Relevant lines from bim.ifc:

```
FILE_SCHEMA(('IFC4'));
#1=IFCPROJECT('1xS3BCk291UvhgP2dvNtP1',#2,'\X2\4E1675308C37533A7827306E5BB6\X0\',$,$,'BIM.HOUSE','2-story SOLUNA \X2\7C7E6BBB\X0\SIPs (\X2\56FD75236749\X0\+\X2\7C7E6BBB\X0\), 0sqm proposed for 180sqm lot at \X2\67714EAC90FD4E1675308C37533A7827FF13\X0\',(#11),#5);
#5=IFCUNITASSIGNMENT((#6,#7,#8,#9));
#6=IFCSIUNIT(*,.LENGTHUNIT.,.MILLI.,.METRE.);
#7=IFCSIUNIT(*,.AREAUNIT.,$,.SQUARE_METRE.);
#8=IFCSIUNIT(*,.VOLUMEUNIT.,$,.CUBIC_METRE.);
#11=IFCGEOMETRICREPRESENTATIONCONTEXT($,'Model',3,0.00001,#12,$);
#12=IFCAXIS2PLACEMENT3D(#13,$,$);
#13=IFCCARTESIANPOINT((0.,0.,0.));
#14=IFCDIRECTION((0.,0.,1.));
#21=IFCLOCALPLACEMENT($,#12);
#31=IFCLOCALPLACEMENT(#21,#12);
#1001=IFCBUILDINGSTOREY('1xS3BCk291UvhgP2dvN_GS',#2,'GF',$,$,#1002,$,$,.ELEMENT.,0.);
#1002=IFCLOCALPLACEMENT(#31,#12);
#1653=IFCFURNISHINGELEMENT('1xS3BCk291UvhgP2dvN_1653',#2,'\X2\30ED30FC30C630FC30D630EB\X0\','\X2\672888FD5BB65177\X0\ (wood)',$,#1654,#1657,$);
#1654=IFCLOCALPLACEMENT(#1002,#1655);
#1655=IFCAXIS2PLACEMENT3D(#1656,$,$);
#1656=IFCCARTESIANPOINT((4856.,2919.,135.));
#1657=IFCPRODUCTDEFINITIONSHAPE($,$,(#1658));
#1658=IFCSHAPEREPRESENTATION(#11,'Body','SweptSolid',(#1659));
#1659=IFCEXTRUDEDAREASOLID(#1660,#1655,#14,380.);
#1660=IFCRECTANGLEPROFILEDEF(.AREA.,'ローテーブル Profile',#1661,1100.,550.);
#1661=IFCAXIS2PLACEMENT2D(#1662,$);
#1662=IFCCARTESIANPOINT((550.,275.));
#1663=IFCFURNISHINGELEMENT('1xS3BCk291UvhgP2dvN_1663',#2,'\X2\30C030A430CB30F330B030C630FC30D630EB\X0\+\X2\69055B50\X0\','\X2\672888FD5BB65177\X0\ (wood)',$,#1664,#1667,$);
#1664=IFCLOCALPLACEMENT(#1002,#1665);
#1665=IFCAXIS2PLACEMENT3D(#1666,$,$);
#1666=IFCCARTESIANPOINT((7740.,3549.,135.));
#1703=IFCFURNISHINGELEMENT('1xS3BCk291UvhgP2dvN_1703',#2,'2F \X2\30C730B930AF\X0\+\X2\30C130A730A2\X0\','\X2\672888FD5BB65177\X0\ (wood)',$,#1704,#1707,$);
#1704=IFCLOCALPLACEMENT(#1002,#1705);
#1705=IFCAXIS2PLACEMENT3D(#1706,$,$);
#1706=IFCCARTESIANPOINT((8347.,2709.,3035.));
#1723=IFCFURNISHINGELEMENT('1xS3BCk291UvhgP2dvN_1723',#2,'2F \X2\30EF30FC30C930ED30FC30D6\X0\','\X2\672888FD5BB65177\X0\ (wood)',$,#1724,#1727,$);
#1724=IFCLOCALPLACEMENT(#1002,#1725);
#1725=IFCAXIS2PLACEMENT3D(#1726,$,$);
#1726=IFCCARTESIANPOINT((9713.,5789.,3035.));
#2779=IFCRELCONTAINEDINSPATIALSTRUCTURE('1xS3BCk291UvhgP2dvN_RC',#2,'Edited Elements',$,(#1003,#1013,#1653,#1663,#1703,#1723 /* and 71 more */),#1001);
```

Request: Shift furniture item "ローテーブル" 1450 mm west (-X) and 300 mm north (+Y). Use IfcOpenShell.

```python
import ifcopenshell
import ifcopenshell.api.geometry
import ifcopenshell.util.placement
import ifcopenshell.util.unit

model = ifcopenshell.open("bim.ifc")
unit_scale = ifcopenshell.util.unit.calculate_unit_scale(model)

item = model.by_guid("1xS3BCk291UvhgP2dvN_1653")
matrix = ifcopenshell.util.placement.get_local_placement(item.ObjectPlacement)
matrix[0, 3] -= 1.45 / unit_scale
matrix[1, 3] += 0.3 / unit_scale
ifcopenshell.api.geometry.edit_object_placement(model, product=item, matrix=matrix, is_si=False)

print(ifcopenshell.util.placement.get_local_placement(item.ObjectPlacement).round(3) + 0.0)

model.write("bim-out.ifc")
```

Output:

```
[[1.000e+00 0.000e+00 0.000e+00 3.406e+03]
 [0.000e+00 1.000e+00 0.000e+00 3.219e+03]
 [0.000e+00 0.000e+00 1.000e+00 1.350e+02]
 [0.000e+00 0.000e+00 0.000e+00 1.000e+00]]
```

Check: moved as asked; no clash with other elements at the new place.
